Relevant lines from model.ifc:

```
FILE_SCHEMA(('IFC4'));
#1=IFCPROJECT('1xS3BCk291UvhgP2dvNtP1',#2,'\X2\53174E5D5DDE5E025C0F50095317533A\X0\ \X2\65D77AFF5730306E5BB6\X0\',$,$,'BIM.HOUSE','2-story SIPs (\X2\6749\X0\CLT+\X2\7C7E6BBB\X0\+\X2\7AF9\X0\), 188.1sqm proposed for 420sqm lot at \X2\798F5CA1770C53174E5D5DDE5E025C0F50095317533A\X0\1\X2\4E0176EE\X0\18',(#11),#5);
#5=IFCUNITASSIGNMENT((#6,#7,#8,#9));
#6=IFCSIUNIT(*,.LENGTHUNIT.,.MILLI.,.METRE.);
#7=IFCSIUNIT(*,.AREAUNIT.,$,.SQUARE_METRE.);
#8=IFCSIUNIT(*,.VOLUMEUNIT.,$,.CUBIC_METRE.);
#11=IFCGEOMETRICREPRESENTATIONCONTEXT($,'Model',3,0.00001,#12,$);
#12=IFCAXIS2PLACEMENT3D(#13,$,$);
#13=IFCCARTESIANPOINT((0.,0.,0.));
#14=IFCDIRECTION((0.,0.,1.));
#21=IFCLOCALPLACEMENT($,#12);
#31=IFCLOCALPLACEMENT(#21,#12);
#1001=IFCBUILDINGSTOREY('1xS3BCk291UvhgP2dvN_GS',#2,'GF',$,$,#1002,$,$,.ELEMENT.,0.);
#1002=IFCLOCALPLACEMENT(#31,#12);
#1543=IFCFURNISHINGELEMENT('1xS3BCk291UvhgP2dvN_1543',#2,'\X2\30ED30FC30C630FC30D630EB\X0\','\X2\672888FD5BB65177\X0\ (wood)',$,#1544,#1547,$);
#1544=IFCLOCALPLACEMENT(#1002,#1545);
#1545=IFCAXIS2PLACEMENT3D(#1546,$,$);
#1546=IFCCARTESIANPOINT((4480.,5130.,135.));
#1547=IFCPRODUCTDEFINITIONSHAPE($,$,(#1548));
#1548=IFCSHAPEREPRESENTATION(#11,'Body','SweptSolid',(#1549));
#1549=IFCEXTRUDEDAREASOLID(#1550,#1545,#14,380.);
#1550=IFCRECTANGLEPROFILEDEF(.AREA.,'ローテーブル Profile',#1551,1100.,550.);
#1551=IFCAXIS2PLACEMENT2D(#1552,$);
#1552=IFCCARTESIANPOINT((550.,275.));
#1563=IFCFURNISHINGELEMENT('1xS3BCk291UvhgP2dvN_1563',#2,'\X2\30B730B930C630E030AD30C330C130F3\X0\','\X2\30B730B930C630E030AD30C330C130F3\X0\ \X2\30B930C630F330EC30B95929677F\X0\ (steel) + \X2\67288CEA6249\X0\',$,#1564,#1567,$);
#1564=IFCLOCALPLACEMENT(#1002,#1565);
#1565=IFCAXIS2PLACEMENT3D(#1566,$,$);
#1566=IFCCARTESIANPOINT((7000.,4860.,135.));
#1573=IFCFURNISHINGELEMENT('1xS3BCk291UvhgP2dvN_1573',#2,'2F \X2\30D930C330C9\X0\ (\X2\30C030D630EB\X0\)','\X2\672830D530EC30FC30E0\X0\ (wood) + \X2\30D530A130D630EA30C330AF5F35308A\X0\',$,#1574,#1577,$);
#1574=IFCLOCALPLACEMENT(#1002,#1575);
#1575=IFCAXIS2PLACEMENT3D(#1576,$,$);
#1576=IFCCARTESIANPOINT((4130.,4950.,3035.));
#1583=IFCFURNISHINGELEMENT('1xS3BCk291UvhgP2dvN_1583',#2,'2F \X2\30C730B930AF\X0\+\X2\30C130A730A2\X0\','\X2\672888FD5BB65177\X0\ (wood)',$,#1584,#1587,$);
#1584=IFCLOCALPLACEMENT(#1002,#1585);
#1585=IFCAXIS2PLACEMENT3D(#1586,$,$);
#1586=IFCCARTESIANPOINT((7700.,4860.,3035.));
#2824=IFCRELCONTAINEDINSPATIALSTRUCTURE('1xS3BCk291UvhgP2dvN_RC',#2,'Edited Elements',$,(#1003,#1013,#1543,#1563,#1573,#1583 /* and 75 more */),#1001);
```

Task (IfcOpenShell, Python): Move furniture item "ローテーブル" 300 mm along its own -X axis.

```python
import ifcopenshell
import ifcopenshell.api.geometry
import ifcopenshell.util.placement

model = ifcopenshell.open("model.ifc")

item = model.by_guid("1xS3BCk291UvhgP2dvN_1543")
matrix = ifcopenshell.util.placement.get_local_placement(item.ObjectPlacement)
matrix[:3, 3] -= matrix[:3, 0] * 300.0
ifcopenshell.api.geometry.edit_object_placement(model, product=item, matrix=matrix, is_si=False)

print(ifcopenshell.util.placement.get_local_placement(item.ObjectPlacement).round(3) + 0.0)

model.write("model_updated.ifc")
```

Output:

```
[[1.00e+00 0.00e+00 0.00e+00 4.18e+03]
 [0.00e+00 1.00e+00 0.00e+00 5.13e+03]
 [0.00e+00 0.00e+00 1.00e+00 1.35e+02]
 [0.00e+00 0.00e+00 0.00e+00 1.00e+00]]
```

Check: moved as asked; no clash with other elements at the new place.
